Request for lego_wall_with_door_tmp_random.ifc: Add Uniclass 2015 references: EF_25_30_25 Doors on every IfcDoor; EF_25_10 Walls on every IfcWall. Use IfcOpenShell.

First a look at what the model holds.

```python
import ifcopenshell

model = ifcopenshell.open("lego_wall_with_door_tmp_random.ifc")
print(model.schema)
print("classifications:", [c.Name for c in model.by_type("IfcClassification")])
for ifc_class in ("IfcDoor", "IfcRoof", "IfcStair", "IfcWall", "IfcWindow"):
    print(ifc_class, len(model.by_type(ifc_class)))
```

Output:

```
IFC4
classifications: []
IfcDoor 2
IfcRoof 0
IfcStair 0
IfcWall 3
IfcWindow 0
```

```python
import ifcopenshell
import ifcopenshell.api.classification

model = ifcopenshell.open("lego_wall_with_door_tmp_random.ifc")

system = ifcopenshell.api.classification.add_classification(model, classification="Uniclass 2015")

codes = {
    "IfcDoor": ("EF_25_30_25", "Doors"),
    "IfcWall": ("EF_25_10", "Walls"),
}
for ifc_class, (code, name) in codes.items():
    products = model.by_type(ifc_class)
    ifcopenshell.api.classification.add_reference(
        model, products=products, classification=system, identification=code, name=name
    )
    print(code, len(products))

model.write("lego_wall_with_door_tmp_random_edited.ifc")
```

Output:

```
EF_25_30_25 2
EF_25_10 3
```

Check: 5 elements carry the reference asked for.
